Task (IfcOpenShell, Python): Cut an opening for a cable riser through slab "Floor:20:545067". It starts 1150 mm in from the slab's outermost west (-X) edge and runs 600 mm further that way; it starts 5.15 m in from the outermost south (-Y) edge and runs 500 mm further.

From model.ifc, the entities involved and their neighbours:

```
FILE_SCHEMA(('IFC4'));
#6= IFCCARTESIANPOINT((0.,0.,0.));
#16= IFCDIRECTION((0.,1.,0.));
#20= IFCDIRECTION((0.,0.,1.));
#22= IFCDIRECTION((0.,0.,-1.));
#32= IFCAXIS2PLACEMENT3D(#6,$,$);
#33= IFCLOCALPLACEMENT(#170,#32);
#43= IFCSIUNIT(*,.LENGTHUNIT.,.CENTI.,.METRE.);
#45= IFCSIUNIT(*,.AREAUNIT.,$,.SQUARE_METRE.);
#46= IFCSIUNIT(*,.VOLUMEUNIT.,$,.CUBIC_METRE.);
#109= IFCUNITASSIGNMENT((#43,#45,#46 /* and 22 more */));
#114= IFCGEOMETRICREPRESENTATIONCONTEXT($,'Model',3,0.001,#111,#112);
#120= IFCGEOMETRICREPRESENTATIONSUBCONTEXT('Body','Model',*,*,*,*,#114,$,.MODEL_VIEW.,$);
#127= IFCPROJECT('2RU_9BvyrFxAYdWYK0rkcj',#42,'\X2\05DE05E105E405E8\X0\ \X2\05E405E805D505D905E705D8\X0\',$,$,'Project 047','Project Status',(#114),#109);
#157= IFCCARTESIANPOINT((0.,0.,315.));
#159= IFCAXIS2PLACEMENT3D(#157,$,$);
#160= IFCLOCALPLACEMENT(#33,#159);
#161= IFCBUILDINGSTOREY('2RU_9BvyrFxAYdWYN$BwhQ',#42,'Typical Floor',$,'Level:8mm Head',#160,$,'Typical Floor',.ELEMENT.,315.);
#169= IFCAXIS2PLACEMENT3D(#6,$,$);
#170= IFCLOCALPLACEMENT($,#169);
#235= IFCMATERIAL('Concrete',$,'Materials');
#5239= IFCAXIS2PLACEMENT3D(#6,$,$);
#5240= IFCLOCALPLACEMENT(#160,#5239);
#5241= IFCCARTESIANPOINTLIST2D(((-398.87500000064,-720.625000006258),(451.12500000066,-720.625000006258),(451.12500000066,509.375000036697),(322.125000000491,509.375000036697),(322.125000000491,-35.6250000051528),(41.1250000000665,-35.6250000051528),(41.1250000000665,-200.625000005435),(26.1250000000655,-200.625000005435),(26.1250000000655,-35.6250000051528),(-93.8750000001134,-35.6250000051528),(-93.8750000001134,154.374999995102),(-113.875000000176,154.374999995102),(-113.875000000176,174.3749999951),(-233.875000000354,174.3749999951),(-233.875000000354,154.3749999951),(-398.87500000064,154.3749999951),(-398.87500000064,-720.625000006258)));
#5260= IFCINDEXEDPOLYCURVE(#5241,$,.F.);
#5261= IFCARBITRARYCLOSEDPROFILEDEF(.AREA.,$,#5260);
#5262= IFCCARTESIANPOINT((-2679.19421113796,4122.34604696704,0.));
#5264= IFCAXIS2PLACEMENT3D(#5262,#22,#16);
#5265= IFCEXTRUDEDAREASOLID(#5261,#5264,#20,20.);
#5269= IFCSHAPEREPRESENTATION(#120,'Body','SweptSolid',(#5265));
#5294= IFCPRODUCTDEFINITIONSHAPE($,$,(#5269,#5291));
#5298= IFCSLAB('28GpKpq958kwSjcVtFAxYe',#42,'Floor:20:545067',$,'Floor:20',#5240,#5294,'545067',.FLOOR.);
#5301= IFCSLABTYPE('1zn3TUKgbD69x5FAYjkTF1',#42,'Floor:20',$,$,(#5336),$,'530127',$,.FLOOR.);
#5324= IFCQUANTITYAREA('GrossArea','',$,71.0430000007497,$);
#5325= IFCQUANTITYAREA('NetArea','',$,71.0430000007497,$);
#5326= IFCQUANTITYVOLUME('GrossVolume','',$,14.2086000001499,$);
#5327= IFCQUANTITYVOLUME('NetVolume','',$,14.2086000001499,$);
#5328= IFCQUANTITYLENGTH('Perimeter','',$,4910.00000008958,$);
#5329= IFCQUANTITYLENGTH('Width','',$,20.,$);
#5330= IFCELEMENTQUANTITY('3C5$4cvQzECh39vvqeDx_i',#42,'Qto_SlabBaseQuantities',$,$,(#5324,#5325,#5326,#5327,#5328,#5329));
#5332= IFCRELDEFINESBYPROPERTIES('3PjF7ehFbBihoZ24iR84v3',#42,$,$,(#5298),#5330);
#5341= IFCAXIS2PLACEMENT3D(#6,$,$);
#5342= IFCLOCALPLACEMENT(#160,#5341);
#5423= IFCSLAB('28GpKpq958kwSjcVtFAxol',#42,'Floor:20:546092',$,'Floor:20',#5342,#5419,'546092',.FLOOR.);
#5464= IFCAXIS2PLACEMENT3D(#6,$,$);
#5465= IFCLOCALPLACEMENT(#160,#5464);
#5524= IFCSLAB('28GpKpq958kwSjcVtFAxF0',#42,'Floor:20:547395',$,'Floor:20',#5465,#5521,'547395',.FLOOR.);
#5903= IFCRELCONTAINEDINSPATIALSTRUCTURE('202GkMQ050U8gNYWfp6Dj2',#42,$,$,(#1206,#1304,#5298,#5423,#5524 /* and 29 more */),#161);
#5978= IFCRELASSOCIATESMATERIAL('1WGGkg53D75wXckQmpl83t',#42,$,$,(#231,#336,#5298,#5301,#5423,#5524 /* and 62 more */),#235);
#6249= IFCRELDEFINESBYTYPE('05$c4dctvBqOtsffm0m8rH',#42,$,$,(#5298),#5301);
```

```python
import numpy as np
import ifcopenshell
import ifcopenshell.api.feature
import ifcopenshell.api.geometry
import ifcopenshell.api.pset
import ifcopenshell.api.root
import ifcopenshell.geom
import ifcopenshell.util.element
import ifcopenshell.util.placement
import ifcopenshell.util.representation
import ifcopenshell.util.shape
import ifcopenshell.util.unit

model = ifcopenshell.open("model.ifc")
unit_scale = ifcopenshell.util.unit.calculate_unit_scale(model)
area_scale = ifcopenshell.util.unit.calculate_unit_scale(model, "AREAUNIT")
volume_scale = ifcopenshell.util.unit.calculate_unit_scale(model, "VOLUMEUNIT")
settings = ifcopenshell.geom.settings()


def volume(element):
    """Net volume in cubic metres, openings subtracted."""
    shape = ifcopenshell.geom.create_shape(settings, element)
    return ifcopenshell.util.shape.get_volume(shape.geometry)


slab = model.by_guid("28GpKpq958kwSjcVtFAxYe")
before = volume(slab)

# Extent in the slab's own axes, in metres. The edges named are its -X and -Y sides.
slab_shape = ifcopenshell.geom.create_shape(settings, slab)
vertices = ifcopenshell.util.shape.get_vertices(slab_shape.geometry)
x_min, y_min, bottom = vertices.min(axis=0)
top = vertices[:, 2].max()

opening = ifcopenshell.api.root.create_entity(model, ifc_class="IfcOpeningElement", name="Cable riser opening", predefined_type="OPENING")
context = ifcopenshell.util.representation.get_context(model, "Model", "Body", "MODEL_VIEW")
width, depth = 0.6, 0.5
outline = [(0.0, 0.0), (width, 0.0), (width, depth), (0.0, depth), (0.0, 0.0)]
# Overshoot both faces by 50 mm so the cut is clean.
shape = ifcopenshell.api.geometry.add_slab_representation(
    model, context=context, depth=top - bottom + 0.1, polyline=outline
)
ifcopenshell.api.geometry.assign_representation(model, product=opening, representation=shape)

matrix = ifcopenshell.util.placement.get_local_placement(slab.ObjectPlacement)
matrix[:, 3] = matrix @ np.append(np.array([x_min + 1.15, y_min + 5.15, bottom - 0.05]) / unit_scale, 1.0)
ifcopenshell.api.geometry.edit_object_placement(model, product=opening, matrix=matrix, is_si=False)
ifcopenshell.api.feature.add_feature(model, feature=opening, element=slab)

after = volume(slab)

# Update the slab's stored quantities.
qto = model.by_id(ifcopenshell.util.element.get_pset(slab, "Qto_SlabBaseQuantities", should_inherit=False)["id"])
ifcopenshell.api.pset.edit_qto(model, qto=qto, properties={
    "NetArea": after / (top - bottom) / area_scale,
    "NetVolume": after / volume_scale,
})

print(f"slab volume {before:.3f} -> {after:.3f} m3")

model.write("model-out.ifc")
```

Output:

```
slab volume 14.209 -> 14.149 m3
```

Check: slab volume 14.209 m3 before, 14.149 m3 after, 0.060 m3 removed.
